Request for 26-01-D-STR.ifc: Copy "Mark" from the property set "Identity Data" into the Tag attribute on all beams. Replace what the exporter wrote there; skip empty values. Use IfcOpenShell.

First a look at what the model holds.

```python
import ifcopenshell
import ifcopenshell.util.element

model = ifcopenshell.open("26-01-D-STR.ifc")
print(model.schema)
beams = model.by_type("IfcBeam")
print(len(beams), "beams")
for e in beams[:8]:
    source = ifcopenshell.util.element.get_pset(e, "Identity Data", "Mark")
    target = e.Tag
    print(e.id(), repr(source), repr(target), sep=" | ")
```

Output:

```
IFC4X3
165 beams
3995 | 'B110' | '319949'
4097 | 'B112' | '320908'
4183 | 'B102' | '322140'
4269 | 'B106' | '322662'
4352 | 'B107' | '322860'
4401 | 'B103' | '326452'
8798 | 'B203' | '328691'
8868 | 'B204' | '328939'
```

```python
import ifcopenshell
import ifcopenshell.util.element

model = ifcopenshell.open("26-01-D-STR.ifc")

count = 0
for e in model.by_type("IfcBeam"):
    value = ifcopenshell.util.element.get_pset(e, "Identity Data", "Mark")
    current = e.Tag
    if not value or not value.strip() or current == value:
        continue
    e.Tag = value
    count += 1

print(count, "beams updated")

model.write("26-01-D-STR_rev.ifc")
```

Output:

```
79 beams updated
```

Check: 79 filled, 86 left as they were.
